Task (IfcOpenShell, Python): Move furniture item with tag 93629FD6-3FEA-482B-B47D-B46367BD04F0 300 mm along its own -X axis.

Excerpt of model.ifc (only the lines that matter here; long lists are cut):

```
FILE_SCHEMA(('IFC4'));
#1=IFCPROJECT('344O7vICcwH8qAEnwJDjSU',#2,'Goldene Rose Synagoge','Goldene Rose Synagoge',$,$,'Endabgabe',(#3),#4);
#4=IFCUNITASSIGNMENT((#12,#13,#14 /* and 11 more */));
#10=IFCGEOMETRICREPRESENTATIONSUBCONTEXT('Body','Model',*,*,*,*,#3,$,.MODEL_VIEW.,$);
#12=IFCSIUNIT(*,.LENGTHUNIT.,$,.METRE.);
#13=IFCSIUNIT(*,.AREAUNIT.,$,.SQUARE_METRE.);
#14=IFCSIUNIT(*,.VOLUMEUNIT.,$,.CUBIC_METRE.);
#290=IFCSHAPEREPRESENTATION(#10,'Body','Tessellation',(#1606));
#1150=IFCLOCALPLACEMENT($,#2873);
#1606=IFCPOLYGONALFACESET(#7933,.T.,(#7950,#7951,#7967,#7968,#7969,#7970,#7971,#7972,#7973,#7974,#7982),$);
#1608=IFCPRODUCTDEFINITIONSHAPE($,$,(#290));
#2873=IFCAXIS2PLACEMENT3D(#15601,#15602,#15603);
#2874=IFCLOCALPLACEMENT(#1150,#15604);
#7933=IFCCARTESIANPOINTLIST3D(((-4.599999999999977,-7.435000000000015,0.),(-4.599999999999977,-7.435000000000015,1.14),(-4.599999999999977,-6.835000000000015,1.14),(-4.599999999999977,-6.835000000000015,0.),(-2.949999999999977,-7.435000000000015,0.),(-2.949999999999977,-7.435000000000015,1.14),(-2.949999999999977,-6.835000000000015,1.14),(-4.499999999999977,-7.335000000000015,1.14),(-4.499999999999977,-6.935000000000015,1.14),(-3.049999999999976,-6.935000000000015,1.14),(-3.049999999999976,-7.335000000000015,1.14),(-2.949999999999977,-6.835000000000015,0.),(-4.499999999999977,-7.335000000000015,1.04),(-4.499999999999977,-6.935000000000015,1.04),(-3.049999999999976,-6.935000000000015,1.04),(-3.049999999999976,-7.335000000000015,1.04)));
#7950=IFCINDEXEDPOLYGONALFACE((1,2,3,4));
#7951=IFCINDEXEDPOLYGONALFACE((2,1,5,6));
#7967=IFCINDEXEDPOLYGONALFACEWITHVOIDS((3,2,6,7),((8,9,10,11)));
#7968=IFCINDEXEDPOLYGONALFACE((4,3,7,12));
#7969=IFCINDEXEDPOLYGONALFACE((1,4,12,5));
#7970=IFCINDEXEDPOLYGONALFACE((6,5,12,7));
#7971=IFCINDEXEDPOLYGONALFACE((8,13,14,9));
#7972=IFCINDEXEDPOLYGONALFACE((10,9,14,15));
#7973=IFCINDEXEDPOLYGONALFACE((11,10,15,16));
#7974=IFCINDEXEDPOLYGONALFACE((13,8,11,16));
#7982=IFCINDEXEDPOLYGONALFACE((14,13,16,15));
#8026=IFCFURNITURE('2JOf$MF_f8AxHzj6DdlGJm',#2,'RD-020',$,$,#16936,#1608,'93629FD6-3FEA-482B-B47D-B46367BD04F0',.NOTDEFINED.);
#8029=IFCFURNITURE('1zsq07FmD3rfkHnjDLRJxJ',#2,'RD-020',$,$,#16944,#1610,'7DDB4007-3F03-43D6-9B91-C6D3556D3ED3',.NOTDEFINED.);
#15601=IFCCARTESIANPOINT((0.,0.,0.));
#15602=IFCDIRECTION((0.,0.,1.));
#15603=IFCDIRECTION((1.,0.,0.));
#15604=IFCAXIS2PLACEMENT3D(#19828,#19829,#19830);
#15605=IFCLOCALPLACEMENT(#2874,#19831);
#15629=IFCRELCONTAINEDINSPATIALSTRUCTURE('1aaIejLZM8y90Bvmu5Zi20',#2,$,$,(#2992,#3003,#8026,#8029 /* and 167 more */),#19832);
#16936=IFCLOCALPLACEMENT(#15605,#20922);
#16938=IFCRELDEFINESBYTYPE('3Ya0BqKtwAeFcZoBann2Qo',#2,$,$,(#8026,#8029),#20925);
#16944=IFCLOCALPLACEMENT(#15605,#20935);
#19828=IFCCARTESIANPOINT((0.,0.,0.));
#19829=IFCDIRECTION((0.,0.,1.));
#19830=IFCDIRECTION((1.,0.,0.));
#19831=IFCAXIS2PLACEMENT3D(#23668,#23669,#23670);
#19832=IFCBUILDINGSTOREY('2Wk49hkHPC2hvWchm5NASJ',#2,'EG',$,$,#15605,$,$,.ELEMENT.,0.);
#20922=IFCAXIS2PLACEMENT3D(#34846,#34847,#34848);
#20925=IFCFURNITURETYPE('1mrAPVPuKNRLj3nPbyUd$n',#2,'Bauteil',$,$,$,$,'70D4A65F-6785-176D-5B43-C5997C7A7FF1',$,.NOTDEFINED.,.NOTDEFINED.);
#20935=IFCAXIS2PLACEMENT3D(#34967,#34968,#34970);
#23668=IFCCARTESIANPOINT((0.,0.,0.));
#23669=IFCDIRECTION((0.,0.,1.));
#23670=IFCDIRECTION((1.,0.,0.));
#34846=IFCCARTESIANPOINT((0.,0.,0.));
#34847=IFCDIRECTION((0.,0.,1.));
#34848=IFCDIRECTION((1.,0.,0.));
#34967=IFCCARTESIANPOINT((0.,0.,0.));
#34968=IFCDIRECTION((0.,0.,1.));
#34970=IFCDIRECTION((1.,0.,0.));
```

```python
import ifcopenshell
import ifcopenshell.api.geometry
import ifcopenshell.util.placement
import ifcopenshell.util.unit

model = ifcopenshell.open("model.ifc")
unit_scale = ifcopenshell.util.unit.calculate_unit_scale(model)

item = model.by_guid("2JOf$MF_f8AxHzj6DdlGJm")
matrix = ifcopenshell.util.placement.get_local_placement(item.ObjectPlacement)
matrix[:3, 3] -= matrix[:3, 0] * 0.3 / unit_scale
ifcopenshell.api.geometry.edit_object_placement(model, product=item, matrix=matrix, is_si=False)

print(ifcopenshell.util.placement.get_local_placement(item.ObjectPlacement).round(3) + 0.0)

model.write("model_v2.ifc")
```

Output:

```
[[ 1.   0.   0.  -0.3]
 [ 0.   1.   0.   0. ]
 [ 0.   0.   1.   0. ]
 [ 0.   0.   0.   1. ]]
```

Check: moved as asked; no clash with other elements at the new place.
